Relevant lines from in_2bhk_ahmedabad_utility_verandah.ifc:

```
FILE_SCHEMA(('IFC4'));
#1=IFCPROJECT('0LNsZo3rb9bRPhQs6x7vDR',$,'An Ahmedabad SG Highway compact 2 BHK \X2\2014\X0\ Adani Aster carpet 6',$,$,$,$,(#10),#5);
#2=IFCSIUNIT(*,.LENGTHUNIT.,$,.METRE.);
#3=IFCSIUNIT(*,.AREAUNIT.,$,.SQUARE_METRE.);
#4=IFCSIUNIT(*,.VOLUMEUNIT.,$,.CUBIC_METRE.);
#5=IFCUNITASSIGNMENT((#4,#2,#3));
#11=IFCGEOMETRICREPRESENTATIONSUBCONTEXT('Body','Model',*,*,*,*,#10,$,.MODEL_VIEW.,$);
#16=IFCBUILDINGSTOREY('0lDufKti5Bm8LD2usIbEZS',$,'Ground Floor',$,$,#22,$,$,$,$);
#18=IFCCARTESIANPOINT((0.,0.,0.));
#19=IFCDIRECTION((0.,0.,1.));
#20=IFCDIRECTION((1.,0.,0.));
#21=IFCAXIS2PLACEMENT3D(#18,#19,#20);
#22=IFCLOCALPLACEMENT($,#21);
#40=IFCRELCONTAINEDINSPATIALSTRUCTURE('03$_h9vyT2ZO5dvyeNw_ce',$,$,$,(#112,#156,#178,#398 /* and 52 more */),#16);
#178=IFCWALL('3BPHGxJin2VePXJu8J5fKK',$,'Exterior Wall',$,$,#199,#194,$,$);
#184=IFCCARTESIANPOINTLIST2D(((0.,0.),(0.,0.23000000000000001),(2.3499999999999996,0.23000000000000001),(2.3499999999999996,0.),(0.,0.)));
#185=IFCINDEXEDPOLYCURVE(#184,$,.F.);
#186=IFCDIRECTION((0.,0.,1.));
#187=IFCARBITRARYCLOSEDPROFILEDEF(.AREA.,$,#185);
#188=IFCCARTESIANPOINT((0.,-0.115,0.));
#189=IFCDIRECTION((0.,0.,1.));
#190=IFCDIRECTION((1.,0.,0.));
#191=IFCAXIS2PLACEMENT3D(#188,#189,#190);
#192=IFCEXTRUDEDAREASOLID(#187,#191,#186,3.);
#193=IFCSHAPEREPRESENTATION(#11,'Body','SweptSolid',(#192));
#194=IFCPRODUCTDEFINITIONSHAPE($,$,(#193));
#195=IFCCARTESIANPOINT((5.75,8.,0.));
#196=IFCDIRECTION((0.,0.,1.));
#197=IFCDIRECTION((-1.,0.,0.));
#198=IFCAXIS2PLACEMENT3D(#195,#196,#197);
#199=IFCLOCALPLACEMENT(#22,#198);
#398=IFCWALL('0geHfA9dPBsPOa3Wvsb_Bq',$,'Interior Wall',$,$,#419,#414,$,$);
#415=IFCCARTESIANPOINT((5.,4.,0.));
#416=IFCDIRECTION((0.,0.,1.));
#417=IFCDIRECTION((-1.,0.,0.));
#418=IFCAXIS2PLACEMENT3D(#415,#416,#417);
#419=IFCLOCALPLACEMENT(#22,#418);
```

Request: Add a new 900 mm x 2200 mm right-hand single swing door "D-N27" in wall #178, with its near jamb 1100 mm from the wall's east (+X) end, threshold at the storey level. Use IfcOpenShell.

```python
import numpy as np
import ifcopenshell
import ifcopenshell.api.feature
import ifcopenshell.api.geometry
import ifcopenshell.api.root
import ifcopenshell.api.spatial
import ifcopenshell.geom
import ifcopenshell.util.element
import ifcopenshell.util.placement
import ifcopenshell.util.representation
import ifcopenshell.util.shape
import ifcopenshell.util.unit

model = ifcopenshell.open("in_2bhk_ahmedabad_utility_verandah.ifc")
unit_scale = ifcopenshell.util.unit.calculate_unit_scale(model)
settings = ifcopenshell.geom.settings()


def volume(element):
    """Net volume in cubic metres, openings subtracted."""
    shape = ifcopenshell.geom.create_shape(settings, element)
    return ifcopenshell.util.shape.get_volume(shape.geometry)


wall = model.by_guid("3BPHGxJin2VePXJu8J5fKK")
storey = ifcopenshell.util.element.get_container(wall, ifc_class="IfcBuildingStorey")
context = ifcopenshell.util.representation.get_context(model, "Model", "Body", "MODEL_VIEW")
before = volume(wall)

width, height, from_end, sill = 0.9, 2.2, 1.1, 0.0  # metres

# The wall runs along its own X axis, and the end named is its -X end.
wall_shape = ifcopenshell.geom.create_shape(settings, wall)
x, y, z = ifcopenshell.util.shape.get_vertices(wall_shape.geometry).T
start = x.min() + from_end
face, thickness = float(y.min()), float(y.max() - y.min())
wall_matrix = ifcopenshell.util.placement.get_local_placement(wall.ObjectPlacement)
level = ifcopenshell.util.placement.get_local_placement(storey.ObjectPlacement)[2, 3]


def in_wall(x, y):
    """Placement at x, y metres in the wall's axes, at sill height."""
    matrix = wall_matrix.copy()
    matrix[:, 3] = wall_matrix @ np.array([x / unit_scale, y / unit_scale, 0.0, 1.0])
    matrix[2, 3] = level + sill / unit_scale
    return matrix


# Opening: a box that overshoots both wall faces by 50 mm.
opening = ifcopenshell.api.root.create_entity(model, ifc_class="IfcOpeningElement", predefined_type="OPENING")
box = ifcopenshell.api.geometry.add_wall_representation(
    model, context=context, length=width, height=height, thickness=thickness + 0.1
)
ifcopenshell.api.geometry.assign_representation(model, product=opening, representation=box)
ifcopenshell.api.geometry.edit_object_placement(model, product=opening, matrix=in_wall(start, face - 0.05), is_si=False)
ifcopenshell.api.feature.add_feature(model, feature=opening, element=wall)

door = ifcopenshell.api.root.create_entity(model, ifc_class="IfcDoor", name="D-N27", predefined_type="DOOR")
door.OverallWidth, door.OverallHeight = width / unit_scale, height / unit_scale
door.OperationType = "SINGLE_SWING_RIGHT"
body = ifcopenshell.api.geometry.add_door_representation(
    model,
    context=context,
    overall_width=door.OverallWidth,
    overall_height=door.OverallHeight,
    operation_type="SINGLE_SWING_RIGHT",
    lining_properties={"LiningDepth": thickness / unit_scale, "ThresholdDepth": thickness / unit_scale},
)
ifcopenshell.api.geometry.assign_representation(model, product=door, representation=body)
ifcopenshell.api.spatial.assign_container(model, products=[door], relating_structure=storey)
ifcopenshell.api.feature.add_filling(model, opening=opening, element=door)

# The lining spans the wall, so the door starts at the wall face.
ifcopenshell.api.geometry.edit_object_placement(model, product=door, matrix=in_wall(start, face), is_si=False)

after = volume(wall)

print(f"wall volume {before:.3f} -> {after:.3f} m3")

model.write("in_2bhk_ahmedabad_utility_verandah_edited.ifc")
```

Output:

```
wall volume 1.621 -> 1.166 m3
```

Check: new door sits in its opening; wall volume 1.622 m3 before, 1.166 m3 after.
